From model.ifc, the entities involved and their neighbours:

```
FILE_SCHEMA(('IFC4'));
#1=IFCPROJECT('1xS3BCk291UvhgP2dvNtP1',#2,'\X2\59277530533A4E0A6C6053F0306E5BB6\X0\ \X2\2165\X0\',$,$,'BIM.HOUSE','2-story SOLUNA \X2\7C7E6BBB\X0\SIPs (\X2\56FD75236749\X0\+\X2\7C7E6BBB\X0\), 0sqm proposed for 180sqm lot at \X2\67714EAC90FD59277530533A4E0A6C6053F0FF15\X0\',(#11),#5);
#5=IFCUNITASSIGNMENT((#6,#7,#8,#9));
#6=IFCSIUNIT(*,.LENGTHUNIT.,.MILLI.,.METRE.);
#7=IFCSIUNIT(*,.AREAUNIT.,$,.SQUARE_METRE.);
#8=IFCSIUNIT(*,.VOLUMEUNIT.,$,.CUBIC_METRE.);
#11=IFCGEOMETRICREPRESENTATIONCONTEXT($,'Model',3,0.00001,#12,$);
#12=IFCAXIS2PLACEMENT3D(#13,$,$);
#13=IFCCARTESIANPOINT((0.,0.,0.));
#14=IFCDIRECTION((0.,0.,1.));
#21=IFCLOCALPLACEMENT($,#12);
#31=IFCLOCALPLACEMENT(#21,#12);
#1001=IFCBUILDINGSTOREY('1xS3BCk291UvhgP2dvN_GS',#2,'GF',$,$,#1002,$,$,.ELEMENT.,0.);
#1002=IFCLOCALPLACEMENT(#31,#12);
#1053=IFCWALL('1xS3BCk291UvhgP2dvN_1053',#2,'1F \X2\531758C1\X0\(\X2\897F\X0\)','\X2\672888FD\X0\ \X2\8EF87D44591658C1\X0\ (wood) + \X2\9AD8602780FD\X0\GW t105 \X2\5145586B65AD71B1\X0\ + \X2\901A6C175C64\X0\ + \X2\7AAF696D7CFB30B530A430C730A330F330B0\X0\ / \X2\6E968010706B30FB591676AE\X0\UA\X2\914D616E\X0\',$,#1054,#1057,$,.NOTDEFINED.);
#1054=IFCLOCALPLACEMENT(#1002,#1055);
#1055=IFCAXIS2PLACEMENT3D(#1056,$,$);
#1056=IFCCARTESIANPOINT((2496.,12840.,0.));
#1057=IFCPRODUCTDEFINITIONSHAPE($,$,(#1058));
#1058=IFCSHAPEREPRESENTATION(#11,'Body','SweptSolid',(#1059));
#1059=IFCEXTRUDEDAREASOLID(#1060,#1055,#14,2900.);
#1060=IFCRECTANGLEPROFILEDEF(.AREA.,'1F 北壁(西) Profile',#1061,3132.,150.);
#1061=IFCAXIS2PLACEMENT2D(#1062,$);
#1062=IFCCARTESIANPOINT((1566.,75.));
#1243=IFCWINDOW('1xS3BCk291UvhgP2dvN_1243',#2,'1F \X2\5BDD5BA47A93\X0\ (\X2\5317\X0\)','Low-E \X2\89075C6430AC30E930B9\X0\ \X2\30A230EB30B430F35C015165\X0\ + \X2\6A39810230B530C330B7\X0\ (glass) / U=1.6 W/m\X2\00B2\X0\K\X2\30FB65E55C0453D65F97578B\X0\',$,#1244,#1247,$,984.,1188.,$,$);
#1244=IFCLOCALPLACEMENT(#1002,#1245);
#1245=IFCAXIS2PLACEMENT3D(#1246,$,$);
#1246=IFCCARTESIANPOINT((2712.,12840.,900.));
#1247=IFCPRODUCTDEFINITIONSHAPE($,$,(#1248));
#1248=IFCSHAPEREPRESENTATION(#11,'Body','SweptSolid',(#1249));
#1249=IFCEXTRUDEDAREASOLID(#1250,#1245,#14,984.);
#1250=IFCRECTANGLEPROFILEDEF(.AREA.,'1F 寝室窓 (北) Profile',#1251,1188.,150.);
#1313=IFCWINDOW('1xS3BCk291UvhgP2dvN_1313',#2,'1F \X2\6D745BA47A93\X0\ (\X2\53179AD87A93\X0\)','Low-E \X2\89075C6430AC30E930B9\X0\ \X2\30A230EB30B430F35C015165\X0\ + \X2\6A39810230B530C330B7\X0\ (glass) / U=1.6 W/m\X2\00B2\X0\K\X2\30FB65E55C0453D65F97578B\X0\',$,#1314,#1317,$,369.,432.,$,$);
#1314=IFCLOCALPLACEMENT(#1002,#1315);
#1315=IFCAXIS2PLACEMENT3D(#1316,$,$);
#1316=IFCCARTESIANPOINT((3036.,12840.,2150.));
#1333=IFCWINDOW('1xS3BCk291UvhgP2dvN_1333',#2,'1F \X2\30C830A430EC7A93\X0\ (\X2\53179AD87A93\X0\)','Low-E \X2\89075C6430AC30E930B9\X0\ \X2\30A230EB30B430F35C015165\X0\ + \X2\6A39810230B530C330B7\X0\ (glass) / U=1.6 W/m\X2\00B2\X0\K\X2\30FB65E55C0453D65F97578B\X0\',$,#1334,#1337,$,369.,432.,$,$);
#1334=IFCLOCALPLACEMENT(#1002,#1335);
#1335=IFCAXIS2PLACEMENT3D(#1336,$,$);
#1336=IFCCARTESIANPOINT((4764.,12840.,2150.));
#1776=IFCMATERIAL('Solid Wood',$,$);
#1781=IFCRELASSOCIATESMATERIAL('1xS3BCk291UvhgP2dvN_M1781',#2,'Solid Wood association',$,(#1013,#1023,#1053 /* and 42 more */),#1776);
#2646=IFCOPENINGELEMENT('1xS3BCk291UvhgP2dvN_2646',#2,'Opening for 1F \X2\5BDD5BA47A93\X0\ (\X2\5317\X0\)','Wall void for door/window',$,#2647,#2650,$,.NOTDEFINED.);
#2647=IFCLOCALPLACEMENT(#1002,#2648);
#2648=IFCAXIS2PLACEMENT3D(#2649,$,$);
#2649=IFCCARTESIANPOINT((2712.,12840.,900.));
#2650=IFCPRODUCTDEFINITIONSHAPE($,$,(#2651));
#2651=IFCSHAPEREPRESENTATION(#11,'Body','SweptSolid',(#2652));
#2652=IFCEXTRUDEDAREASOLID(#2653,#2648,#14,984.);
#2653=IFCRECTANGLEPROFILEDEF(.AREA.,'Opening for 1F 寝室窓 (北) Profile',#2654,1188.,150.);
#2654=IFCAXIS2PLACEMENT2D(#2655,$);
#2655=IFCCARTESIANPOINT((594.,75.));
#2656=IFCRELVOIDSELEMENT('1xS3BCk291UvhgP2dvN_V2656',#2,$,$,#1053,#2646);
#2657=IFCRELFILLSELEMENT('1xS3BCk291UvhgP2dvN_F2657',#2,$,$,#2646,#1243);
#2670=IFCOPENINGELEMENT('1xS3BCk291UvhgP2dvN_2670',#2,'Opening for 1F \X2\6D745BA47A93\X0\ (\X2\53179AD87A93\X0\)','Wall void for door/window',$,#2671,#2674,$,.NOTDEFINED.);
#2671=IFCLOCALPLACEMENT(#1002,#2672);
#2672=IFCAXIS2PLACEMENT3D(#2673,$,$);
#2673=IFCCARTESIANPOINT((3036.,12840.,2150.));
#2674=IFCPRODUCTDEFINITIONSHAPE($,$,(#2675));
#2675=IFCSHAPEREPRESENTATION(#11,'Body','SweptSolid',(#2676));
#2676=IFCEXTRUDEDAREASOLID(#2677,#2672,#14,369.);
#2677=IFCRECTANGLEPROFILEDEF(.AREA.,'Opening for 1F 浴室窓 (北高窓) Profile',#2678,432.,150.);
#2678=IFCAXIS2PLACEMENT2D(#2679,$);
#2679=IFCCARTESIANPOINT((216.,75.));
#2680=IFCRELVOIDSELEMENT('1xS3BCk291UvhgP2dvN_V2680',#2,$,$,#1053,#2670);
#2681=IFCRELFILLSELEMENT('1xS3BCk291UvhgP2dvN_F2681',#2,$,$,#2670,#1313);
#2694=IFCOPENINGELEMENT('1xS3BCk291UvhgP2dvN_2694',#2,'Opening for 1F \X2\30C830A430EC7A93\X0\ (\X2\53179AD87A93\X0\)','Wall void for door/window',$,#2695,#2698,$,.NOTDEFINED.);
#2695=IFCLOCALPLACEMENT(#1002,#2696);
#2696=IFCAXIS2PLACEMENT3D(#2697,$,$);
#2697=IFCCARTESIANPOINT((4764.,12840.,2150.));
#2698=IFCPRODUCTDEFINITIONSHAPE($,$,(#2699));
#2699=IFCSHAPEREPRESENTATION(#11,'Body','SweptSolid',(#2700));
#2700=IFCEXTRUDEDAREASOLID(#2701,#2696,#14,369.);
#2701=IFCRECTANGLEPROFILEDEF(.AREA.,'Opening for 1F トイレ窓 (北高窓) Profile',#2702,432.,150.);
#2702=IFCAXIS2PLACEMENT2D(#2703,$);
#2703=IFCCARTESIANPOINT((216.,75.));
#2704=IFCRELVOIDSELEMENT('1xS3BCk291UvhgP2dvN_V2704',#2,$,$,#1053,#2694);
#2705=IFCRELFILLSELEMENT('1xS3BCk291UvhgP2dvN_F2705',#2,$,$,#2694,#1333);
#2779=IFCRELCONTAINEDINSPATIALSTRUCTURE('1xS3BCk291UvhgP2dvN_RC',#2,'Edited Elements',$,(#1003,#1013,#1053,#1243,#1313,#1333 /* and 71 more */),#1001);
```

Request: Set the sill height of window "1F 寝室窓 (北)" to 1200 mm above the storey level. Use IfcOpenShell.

```python
import numpy as np
import ifcopenshell
import ifcopenshell.api.geometry
import ifcopenshell.geom
import ifcopenshell.util.element
import ifcopenshell.util.placement
import ifcopenshell.util.shape
import ifcopenshell.util.unit

model = ifcopenshell.open("model.ifc")
unit_scale = ifcopenshell.util.unit.calculate_unit_scale(model)

window = model.by_guid("1xS3BCk291UvhgP2dvN_1243")
opening = window.FillsVoids[0].RelatingOpeningElement
storey = ifcopenshell.util.element.get_container(window, ifc_class="IfcBuildingStorey")
level = ifcopenshell.util.placement.get_local_placement(storey.ObjectPlacement)[2, 3]

# The opening's origin need not be at the sill, so measure its lowest point.
shape = ifcopenshell.geom.create_shape(ifcopenshell.geom.settings(), opening)
bottom = ifcopenshell.util.shape.get_shape_bottom_elevation(shape, shape.geometry) / unit_scale
dz = level + 1.2 / unit_scale - bottom

shift = np.array([0.0, 0.0, dz])
# The window is not placed relative to its opening, so move both.
for product in (opening, window):
    matrix = ifcopenshell.util.placement.get_local_placement(product.ObjectPlacement)
    matrix[:3, 3] += shift
    ifcopenshell.api.geometry.edit_object_placement(model, product=product, matrix=matrix, is_si=False)

print(f"moved by {dz * unit_scale:+.3f} m")

model.write("model_edited.ifc")
```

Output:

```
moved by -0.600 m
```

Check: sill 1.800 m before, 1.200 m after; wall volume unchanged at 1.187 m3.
